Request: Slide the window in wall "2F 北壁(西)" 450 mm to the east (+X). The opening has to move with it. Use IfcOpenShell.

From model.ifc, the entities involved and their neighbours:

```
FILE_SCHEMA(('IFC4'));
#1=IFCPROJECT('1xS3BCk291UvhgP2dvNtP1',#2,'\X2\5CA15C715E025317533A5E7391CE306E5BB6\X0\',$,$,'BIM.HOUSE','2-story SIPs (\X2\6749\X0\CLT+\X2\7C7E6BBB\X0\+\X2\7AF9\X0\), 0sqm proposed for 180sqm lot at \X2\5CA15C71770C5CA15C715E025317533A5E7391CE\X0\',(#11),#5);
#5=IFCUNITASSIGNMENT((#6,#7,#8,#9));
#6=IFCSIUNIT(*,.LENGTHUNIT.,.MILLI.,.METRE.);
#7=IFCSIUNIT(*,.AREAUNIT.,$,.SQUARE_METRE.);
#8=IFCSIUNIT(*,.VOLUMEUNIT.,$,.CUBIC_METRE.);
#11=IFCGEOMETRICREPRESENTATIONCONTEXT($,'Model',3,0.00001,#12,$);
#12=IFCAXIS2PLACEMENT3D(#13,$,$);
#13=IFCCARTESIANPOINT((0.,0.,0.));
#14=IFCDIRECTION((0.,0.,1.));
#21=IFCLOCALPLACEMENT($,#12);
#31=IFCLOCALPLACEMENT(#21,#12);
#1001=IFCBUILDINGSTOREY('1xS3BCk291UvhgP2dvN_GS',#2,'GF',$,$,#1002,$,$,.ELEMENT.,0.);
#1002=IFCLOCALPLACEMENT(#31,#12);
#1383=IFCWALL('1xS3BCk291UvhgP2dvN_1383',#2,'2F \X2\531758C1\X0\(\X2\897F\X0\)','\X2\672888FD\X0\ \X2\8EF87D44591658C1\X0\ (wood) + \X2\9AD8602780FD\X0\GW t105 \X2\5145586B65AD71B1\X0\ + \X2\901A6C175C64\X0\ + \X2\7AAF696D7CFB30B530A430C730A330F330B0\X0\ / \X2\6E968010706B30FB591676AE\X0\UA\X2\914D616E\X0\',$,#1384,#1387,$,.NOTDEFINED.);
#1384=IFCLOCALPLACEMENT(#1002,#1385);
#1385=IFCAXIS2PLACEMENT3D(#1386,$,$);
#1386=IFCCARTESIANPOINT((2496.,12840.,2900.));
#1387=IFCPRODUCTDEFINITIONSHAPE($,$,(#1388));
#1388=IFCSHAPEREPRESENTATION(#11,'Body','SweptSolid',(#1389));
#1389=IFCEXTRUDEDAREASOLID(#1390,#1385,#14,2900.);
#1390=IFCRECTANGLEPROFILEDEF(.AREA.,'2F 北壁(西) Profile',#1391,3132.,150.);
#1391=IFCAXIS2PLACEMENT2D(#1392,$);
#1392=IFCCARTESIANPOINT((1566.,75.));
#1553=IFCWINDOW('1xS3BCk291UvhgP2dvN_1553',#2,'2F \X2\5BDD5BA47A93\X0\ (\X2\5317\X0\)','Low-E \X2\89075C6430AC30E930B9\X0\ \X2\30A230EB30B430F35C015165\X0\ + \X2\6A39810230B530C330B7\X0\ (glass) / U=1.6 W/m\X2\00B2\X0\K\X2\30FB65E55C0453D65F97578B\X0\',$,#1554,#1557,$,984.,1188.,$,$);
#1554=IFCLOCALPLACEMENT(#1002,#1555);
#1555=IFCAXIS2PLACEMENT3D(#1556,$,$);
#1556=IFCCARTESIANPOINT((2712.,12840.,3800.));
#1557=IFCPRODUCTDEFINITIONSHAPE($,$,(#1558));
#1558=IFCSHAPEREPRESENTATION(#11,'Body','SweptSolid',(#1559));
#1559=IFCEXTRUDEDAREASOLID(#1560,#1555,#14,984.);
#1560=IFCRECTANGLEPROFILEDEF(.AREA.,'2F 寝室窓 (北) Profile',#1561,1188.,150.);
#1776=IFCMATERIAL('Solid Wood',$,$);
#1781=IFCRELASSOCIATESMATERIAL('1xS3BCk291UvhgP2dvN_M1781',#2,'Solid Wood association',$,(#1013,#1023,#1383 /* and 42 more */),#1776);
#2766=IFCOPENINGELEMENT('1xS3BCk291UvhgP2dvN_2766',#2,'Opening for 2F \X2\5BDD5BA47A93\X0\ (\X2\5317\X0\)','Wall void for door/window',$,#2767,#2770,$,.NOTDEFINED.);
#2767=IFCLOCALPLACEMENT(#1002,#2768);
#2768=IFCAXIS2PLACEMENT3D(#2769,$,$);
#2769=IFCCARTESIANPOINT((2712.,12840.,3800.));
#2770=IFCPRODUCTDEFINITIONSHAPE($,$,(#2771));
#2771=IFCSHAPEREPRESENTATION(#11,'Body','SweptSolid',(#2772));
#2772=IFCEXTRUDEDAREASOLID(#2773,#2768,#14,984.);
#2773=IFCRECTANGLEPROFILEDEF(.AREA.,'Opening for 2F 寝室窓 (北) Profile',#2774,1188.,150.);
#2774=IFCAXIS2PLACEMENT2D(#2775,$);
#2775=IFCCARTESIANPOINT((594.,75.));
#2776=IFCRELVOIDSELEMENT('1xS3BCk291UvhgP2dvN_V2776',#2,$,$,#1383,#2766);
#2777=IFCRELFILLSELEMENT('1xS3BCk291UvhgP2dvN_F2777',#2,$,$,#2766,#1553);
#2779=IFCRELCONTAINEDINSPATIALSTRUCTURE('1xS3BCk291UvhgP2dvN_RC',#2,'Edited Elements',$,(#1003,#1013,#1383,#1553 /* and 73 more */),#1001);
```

```python
import ifcopenshell
import ifcopenshell.api.geometry
import ifcopenshell.util.placement
import ifcopenshell.util.unit

model = ifcopenshell.open("model.ifc")
unit_scale = ifcopenshell.util.unit.calculate_unit_scale(model)

window = model.by_guid("1xS3BCk291UvhgP2dvN_1553")
opening = window.FillsVoids[0].RelatingOpeningElement
wall = opening.VoidsElements[0].RelatingBuildingElement

wall_matrix = ifcopenshell.util.placement.get_local_placement(wall.ObjectPlacement)
shift = wall_matrix[:3, 0] * 0.45 / unit_scale
before = ifcopenshell.util.placement.get_local_placement(window.ObjectPlacement)[:3, 3].copy()

# The window is not placed relative to its opening, so move both.
for product in (opening, window):
    matrix = ifcopenshell.util.placement.get_local_placement(product.ObjectPlacement)
    matrix[:3, 3] += shift
    ifcopenshell.api.geometry.edit_object_placement(model, product=product, matrix=matrix, is_si=False)

after = ifcopenshell.util.placement.get_local_placement(window.ObjectPlacement)[:3, 3]
print("window moved by", (after - before).round(3) + 0.0)

model.write("model-out.ifc")
```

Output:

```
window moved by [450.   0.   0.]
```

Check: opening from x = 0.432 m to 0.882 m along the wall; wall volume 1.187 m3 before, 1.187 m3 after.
